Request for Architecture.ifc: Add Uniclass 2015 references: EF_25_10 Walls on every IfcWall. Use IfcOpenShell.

First a look at what the model holds.

```python
import ifcopenshell

model = ifcopenshell.open("Architecture.ifc")
print(model.schema)
print("classifications:", [c.Name for c in model.by_type("IfcClassification")])
for ifc_class in ("IfcDoor", "IfcRoof", "IfcStair", "IfcWall", "IfcWindow"):
    print(ifc_class, len(model.by_type(ifc_class)))
```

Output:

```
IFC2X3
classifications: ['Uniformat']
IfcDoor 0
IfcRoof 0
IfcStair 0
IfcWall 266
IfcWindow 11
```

```python
import ifcopenshell
import ifcopenshell.api.classification

model = ifcopenshell.open("Architecture.ifc")

# IFC2X3 requires Source and Edition and has no link from the project to the system.
system = model.create_entity("IfcClassification", Source="NBS", Edition="2015", Name="Uniclass 2015")

codes = {
    "IfcWall": ("EF_25_10", "Walls"),
}
for ifc_class, (code, name) in codes.items():
    products = model.by_type(ifc_class)
    ifcopenshell.api.classification.add_reference(
        model, products=products, classification=system, identification=code, name=name
    )
    print(code, len(products))

model.write("Architecture_edited.ifc")
```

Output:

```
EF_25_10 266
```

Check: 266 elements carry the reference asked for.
